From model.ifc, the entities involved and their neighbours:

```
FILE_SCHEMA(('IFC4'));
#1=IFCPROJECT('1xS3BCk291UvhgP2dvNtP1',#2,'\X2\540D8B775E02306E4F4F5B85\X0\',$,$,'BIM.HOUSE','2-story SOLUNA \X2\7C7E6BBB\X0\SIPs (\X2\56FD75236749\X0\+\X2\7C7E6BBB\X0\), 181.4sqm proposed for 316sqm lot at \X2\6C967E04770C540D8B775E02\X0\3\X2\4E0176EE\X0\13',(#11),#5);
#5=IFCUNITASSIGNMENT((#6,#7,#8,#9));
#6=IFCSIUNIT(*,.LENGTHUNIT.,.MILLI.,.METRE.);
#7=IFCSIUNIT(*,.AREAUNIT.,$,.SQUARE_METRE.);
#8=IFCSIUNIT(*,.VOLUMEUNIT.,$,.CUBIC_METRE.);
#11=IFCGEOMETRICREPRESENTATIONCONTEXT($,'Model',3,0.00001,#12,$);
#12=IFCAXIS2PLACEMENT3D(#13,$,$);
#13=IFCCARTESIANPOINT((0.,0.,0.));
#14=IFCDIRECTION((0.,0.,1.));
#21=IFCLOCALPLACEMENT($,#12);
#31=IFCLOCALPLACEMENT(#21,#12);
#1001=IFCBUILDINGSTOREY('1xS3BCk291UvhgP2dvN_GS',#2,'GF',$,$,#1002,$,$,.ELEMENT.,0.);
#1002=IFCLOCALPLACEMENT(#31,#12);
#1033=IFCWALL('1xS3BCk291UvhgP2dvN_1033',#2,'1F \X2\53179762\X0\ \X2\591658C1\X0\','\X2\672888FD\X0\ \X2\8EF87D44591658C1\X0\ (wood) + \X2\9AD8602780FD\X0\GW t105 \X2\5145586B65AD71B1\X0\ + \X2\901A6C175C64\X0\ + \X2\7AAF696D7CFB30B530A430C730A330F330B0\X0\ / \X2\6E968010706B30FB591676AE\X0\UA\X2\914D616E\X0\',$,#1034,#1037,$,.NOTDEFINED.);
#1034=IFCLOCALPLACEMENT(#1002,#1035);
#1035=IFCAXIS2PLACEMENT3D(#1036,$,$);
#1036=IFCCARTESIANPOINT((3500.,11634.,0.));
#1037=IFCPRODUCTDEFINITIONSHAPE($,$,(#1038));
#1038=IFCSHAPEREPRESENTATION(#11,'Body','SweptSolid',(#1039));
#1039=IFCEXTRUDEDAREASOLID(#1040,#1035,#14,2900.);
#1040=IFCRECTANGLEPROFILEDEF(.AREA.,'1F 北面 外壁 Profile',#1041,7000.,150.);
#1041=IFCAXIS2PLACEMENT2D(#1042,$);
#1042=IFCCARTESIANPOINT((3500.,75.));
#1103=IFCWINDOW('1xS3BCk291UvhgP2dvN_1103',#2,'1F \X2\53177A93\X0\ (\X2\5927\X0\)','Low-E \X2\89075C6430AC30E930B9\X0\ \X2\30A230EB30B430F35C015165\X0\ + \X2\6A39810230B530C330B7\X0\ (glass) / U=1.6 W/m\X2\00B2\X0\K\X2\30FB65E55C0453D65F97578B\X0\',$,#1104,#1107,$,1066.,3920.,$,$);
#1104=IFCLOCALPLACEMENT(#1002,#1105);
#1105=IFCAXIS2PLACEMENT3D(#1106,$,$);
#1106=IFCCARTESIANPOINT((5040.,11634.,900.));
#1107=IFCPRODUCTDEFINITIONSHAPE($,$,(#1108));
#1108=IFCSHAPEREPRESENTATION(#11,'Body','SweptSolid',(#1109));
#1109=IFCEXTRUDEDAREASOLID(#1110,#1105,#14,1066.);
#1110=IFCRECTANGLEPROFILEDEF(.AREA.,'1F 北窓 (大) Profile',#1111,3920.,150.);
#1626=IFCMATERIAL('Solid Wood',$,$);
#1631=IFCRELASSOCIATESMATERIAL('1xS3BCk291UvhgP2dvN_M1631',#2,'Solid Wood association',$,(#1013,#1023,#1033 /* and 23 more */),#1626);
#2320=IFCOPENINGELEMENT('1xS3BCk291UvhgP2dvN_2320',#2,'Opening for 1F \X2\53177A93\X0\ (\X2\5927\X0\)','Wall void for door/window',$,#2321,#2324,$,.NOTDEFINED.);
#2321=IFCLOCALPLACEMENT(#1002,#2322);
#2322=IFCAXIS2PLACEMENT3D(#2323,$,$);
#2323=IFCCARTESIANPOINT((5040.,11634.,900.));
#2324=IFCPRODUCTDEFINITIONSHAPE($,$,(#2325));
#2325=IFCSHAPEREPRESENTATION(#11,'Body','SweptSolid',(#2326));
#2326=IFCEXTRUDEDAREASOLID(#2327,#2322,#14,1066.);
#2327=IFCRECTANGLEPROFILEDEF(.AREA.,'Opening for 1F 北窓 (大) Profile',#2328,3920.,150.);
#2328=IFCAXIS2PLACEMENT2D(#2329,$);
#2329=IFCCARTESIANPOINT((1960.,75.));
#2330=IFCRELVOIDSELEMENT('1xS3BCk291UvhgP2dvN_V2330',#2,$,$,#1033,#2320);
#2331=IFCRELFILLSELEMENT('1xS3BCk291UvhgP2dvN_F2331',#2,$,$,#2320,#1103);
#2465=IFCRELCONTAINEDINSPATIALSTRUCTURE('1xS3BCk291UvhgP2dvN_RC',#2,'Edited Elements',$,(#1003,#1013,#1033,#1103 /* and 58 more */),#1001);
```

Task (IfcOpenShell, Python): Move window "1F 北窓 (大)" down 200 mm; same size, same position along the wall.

```python
import numpy as np
import ifcopenshell
import ifcopenshell.api.geometry
import ifcopenshell.util.placement
import ifcopenshell.util.unit

model = ifcopenshell.open("model.ifc")
unit_scale = ifcopenshell.util.unit.calculate_unit_scale(model)

window = model.by_guid("1xS3BCk291UvhgP2dvN_1103")
opening = window.FillsVoids[0].RelatingOpeningElement
dz = -0.2 / unit_scale

shift = np.array([0.0, 0.0, dz])
# The window is not placed relative to its opening, so move both.
for product in (opening, window):
    matrix = ifcopenshell.util.placement.get_local_placement(product.ObjectPlacement)
    matrix[:3, 3] += shift
    ifcopenshell.api.geometry.edit_object_placement(model, product=product, matrix=matrix, is_si=False)

print(f"moved by {dz * unit_scale:+.3f} m")

model.write("model_edited.ifc")
```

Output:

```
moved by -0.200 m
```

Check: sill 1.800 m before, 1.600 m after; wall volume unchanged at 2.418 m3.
